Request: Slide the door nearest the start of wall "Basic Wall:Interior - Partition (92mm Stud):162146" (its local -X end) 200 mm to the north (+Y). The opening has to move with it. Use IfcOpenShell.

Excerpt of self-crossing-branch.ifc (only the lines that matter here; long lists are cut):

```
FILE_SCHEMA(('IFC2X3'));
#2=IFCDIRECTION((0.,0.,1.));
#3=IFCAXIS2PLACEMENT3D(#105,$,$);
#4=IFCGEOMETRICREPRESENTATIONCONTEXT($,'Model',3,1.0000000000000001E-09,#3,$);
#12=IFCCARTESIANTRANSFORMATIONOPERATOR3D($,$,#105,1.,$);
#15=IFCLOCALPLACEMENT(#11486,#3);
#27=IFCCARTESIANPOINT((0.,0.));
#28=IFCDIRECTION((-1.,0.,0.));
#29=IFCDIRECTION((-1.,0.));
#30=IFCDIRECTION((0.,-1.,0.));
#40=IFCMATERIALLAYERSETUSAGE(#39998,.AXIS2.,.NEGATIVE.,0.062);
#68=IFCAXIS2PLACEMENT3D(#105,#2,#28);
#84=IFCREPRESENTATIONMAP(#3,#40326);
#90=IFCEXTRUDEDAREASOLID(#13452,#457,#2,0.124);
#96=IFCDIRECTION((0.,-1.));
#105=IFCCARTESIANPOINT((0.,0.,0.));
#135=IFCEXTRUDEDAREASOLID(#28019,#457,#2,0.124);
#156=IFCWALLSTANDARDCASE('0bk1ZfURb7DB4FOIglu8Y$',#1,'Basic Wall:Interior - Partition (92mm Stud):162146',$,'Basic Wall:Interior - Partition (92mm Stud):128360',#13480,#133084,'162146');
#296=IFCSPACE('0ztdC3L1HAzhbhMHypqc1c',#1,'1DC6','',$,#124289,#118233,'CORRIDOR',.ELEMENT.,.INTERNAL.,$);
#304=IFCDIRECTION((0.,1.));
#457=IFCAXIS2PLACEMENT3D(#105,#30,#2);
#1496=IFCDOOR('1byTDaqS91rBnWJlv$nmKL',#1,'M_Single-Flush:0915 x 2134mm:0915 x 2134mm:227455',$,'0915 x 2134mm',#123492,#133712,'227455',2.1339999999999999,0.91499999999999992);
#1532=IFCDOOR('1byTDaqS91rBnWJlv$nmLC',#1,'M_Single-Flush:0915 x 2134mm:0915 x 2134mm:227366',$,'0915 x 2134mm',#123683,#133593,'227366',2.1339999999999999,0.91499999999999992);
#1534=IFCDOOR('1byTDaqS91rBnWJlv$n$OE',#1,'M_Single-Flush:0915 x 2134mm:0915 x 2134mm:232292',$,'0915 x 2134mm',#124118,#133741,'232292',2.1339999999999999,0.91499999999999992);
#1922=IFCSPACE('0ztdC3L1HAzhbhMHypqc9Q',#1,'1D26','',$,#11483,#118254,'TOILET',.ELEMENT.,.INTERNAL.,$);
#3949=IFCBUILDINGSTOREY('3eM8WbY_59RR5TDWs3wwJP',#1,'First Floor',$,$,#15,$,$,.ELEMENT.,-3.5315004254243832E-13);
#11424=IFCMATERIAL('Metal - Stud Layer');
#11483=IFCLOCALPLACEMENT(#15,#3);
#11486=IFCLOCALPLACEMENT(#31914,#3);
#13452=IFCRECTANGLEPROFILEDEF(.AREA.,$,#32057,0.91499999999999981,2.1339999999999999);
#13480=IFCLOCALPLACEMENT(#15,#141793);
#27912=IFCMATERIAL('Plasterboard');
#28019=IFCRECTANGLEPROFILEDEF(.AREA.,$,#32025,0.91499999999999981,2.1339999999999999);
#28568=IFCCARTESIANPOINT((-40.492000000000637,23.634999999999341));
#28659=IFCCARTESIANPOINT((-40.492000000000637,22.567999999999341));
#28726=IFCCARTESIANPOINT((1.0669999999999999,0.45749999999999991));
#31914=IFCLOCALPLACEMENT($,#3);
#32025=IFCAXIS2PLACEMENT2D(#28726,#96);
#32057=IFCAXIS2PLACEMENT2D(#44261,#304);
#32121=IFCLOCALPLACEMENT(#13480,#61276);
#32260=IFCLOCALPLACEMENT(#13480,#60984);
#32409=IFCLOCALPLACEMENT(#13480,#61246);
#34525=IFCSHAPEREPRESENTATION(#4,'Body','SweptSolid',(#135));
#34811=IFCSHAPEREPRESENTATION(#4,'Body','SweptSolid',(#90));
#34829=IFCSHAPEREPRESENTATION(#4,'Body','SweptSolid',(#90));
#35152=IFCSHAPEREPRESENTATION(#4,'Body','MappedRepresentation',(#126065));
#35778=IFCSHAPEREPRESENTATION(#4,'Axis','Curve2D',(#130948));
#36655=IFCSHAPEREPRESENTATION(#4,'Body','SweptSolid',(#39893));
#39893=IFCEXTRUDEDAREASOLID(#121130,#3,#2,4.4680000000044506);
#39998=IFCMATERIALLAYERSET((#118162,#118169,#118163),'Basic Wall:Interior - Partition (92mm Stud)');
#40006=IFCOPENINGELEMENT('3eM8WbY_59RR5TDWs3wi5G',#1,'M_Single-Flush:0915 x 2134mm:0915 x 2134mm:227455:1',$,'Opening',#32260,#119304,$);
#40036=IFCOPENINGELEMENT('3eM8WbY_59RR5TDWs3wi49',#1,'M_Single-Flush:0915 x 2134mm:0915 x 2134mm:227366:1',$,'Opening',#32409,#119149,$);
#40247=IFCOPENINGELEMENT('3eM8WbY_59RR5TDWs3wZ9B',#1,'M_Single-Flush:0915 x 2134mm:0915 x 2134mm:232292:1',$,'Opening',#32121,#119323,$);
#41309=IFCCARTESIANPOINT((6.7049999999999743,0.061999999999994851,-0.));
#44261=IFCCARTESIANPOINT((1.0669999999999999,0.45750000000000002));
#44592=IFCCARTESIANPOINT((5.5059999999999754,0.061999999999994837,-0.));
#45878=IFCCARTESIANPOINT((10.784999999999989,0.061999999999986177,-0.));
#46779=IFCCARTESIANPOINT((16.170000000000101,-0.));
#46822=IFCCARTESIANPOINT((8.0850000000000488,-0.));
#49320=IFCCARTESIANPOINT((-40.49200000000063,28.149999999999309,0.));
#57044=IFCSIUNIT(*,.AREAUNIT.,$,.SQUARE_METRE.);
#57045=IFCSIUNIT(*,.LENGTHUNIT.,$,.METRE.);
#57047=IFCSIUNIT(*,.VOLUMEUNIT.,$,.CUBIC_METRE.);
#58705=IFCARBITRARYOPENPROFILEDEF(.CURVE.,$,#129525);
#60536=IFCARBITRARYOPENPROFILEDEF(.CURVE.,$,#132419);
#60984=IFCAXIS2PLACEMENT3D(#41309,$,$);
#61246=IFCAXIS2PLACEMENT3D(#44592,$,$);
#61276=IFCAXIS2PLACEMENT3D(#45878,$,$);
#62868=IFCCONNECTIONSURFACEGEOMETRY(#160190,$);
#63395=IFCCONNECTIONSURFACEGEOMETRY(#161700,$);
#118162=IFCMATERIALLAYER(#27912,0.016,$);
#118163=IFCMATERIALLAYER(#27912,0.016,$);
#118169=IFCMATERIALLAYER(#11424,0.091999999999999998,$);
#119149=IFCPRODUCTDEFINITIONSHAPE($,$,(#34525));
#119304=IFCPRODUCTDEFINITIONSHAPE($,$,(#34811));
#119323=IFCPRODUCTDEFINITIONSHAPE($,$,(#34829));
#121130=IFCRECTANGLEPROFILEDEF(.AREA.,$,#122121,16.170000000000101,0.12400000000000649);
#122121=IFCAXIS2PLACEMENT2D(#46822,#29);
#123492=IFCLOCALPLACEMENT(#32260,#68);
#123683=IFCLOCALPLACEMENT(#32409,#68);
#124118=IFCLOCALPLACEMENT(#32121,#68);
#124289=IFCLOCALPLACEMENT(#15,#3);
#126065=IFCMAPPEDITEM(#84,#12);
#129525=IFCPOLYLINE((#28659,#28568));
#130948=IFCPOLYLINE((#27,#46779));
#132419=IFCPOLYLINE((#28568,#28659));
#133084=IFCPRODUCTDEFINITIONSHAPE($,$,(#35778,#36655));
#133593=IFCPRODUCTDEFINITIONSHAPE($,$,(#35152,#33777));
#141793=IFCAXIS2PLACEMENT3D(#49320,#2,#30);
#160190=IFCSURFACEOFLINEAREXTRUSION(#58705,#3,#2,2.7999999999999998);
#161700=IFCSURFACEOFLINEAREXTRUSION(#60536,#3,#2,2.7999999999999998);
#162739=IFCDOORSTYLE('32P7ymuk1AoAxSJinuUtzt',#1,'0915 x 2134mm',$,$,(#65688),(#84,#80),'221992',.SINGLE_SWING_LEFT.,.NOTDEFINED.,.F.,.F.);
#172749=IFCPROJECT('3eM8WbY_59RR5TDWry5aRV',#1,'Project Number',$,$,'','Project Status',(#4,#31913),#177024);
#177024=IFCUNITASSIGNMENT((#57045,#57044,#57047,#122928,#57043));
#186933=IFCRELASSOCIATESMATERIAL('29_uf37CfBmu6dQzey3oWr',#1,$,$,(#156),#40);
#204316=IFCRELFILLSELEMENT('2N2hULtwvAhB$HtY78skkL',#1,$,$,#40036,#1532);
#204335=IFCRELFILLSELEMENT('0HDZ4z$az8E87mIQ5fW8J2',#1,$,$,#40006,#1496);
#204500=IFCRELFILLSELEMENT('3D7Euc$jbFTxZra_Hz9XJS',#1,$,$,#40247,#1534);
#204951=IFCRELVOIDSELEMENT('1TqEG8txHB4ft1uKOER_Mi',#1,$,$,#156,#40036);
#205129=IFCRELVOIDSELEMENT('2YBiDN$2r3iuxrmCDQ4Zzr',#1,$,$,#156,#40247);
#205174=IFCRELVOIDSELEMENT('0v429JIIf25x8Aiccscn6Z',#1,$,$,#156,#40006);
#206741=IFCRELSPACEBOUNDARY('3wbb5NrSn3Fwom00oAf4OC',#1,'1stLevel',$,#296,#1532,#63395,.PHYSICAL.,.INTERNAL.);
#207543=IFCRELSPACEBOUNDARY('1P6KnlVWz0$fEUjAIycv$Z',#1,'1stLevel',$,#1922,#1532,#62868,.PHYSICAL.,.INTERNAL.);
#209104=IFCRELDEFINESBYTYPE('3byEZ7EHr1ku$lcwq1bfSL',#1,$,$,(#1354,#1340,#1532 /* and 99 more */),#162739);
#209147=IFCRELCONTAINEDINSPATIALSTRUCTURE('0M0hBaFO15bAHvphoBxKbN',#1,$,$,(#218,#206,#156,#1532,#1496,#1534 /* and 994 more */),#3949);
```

```python
import numpy as np
import ifcopenshell
import ifcopenshell.api.geometry
import ifcopenshell.util.placement

model = ifcopenshell.open("self-crossing-branch.ifc")

door = model.by_id(1532)
opening = door.FillsVoids[0].RelatingOpeningElement
wall = opening.VoidsElements[0].RelatingBuildingElement

wall_matrix = ifcopenshell.util.placement.get_local_placement(wall.ObjectPlacement)
shift = wall_matrix[:3, 0] * -0.2
before = ifcopenshell.util.placement.get_local_placement(door.ObjectPlacement)[:3, 3].copy()

# The door is placed relative to its opening, so it follows when the opening moves.
matrix = ifcopenshell.util.placement.get_local_placement(opening.ObjectPlacement)
matrix[:3, 3] += shift
ifcopenshell.api.geometry.edit_object_placement(
    model, product=opening, matrix=matrix, is_si=False, should_transform_children=True
)

# Space boundary surfaces are stored in each space's coordinates; move them too.
for rel in door.ProvidesBoundaries:
    if not rel.ConnectionGeometry:
        continue
    surface = rel.ConnectionGeometry.SurfaceOnRelatingElement
    space_matrix = ifcopenshell.util.placement.get_local_placement(rel.RelatingSpace.ObjectPlacement)
    point = np.array(surface.Position.Location.Coordinates) + space_matrix[:3, :3].T @ shift
    surface.Position = model.createIfcAxis2Placement3D(
        model.createIfcCartesianPoint(point.tolist()), surface.Position.Axis, surface.Position.RefDirection
    )

after = ifcopenshell.util.placement.get_local_placement(door.ObjectPlacement)[:3, 3]
print("door moved by", (after - before).round(3) + 0.0)

model.write("self-crossing-branch_v2.ifc")
```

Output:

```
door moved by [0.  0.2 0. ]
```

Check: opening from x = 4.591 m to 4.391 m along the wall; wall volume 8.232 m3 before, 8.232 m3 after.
